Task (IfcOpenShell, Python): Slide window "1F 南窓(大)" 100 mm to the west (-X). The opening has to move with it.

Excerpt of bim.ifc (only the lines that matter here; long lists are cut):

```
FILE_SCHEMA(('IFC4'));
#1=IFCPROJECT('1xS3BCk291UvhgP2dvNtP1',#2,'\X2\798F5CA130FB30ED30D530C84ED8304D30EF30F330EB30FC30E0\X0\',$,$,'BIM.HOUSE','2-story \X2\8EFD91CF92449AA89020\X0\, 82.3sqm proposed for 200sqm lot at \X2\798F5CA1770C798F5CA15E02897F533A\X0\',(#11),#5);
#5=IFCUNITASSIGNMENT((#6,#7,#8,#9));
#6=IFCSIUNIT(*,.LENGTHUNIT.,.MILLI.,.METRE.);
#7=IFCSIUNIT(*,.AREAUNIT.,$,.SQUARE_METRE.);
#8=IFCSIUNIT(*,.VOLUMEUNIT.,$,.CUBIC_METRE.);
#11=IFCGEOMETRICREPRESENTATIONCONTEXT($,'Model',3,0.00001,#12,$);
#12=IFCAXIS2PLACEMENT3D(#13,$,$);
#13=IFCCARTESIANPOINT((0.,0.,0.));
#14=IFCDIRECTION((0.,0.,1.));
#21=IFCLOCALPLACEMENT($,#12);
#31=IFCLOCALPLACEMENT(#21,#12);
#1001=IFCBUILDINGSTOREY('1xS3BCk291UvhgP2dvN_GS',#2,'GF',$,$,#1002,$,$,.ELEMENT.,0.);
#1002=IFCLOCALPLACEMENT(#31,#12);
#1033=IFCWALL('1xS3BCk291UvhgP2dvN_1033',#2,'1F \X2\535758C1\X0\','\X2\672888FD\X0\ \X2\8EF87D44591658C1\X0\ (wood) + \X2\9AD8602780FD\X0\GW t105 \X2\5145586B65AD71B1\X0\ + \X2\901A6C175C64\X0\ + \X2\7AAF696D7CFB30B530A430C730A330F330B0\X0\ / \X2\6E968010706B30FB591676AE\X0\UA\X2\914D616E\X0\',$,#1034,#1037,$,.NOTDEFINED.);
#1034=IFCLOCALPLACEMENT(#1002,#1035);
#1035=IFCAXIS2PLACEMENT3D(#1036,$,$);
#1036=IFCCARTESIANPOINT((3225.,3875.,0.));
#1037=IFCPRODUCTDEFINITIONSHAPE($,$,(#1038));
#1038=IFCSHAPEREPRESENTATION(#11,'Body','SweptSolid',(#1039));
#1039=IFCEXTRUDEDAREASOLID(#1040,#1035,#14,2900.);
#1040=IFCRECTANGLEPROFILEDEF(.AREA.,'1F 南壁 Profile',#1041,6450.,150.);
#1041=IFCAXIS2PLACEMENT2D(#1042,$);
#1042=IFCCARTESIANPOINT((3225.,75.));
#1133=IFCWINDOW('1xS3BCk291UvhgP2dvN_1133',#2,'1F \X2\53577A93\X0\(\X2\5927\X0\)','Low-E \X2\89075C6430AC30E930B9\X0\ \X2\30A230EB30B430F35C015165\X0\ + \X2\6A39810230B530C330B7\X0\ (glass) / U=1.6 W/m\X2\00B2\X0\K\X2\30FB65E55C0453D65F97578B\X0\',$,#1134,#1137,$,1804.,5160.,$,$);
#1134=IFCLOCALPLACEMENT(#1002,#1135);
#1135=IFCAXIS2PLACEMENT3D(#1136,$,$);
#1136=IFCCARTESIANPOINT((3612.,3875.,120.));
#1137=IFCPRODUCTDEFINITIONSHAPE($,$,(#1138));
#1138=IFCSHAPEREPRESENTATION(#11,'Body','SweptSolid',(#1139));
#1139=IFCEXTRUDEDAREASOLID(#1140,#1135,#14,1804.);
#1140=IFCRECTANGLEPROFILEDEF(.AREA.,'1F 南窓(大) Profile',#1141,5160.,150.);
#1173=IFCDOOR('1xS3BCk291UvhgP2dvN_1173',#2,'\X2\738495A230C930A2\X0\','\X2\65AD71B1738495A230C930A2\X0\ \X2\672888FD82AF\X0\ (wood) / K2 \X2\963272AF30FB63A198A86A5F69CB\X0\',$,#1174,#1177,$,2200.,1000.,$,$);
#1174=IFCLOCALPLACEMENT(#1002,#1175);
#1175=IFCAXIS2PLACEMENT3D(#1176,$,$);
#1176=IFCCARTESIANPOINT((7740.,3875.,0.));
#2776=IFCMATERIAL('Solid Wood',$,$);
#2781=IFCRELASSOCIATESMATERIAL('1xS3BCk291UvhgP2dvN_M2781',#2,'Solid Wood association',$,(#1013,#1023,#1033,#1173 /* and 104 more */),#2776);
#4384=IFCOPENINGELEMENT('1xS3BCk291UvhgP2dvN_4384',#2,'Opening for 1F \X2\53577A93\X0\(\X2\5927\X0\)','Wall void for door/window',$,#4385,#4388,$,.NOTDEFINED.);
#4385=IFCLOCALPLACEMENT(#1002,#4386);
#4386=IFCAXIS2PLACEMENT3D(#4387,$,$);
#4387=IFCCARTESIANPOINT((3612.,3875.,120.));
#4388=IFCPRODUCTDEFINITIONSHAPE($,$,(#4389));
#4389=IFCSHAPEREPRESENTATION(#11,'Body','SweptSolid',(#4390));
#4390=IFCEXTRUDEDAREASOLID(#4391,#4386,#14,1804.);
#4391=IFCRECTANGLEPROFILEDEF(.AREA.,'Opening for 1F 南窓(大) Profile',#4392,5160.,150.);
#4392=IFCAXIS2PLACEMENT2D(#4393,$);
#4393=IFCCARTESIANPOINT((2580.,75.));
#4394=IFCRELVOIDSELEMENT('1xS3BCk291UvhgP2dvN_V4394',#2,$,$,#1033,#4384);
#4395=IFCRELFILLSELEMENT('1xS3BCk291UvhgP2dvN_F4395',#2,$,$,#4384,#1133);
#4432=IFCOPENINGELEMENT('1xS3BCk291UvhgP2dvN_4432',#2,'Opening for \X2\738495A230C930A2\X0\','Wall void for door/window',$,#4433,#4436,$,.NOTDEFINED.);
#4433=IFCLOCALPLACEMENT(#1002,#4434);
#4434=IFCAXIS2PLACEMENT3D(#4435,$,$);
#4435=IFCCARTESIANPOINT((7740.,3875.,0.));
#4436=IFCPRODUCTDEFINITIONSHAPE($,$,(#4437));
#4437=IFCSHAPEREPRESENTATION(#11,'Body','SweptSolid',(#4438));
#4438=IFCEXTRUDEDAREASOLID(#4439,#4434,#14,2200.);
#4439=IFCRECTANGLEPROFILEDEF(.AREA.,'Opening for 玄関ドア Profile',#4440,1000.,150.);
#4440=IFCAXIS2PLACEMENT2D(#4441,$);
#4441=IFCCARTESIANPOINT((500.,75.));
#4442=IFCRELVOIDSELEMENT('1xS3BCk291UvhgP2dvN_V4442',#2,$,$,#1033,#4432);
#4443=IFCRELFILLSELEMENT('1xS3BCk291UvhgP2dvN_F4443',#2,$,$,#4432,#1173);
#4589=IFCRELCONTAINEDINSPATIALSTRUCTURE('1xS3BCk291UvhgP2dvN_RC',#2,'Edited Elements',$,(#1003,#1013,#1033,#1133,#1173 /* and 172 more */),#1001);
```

```python
import ifcopenshell
import ifcopenshell.api.geometry
import ifcopenshell.util.placement
import ifcopenshell.util.unit

model = ifcopenshell.open("bim.ifc")
unit_scale = ifcopenshell.util.unit.calculate_unit_scale(model)

window = model.by_guid("1xS3BCk291UvhgP2dvN_1133")
opening = window.FillsVoids[0].RelatingOpeningElement
wall = opening.VoidsElements[0].RelatingBuildingElement

wall_matrix = ifcopenshell.util.placement.get_local_placement(wall.ObjectPlacement)
shift = wall_matrix[:3, 0] * -0.1 / unit_scale
before = ifcopenshell.util.placement.get_local_placement(window.ObjectPlacement)[:3, 3].copy()

# The window is not placed relative to its opening, so move both.
for product in (opening, window):
    matrix = ifcopenshell.util.placement.get_local_placement(product.ObjectPlacement)
    matrix[:3, 3] += shift
    ifcopenshell.api.geometry.edit_object_placement(model, product=product, matrix=matrix, is_si=False)

after = ifcopenshell.util.placement.get_local_placement(window.ObjectPlacement)[:3, 3]
print("window moved by", (after - before).round(3) + 0.0)

model.write("bim_edited.ifc")
```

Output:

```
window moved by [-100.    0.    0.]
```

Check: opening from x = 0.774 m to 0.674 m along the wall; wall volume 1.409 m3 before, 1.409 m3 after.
